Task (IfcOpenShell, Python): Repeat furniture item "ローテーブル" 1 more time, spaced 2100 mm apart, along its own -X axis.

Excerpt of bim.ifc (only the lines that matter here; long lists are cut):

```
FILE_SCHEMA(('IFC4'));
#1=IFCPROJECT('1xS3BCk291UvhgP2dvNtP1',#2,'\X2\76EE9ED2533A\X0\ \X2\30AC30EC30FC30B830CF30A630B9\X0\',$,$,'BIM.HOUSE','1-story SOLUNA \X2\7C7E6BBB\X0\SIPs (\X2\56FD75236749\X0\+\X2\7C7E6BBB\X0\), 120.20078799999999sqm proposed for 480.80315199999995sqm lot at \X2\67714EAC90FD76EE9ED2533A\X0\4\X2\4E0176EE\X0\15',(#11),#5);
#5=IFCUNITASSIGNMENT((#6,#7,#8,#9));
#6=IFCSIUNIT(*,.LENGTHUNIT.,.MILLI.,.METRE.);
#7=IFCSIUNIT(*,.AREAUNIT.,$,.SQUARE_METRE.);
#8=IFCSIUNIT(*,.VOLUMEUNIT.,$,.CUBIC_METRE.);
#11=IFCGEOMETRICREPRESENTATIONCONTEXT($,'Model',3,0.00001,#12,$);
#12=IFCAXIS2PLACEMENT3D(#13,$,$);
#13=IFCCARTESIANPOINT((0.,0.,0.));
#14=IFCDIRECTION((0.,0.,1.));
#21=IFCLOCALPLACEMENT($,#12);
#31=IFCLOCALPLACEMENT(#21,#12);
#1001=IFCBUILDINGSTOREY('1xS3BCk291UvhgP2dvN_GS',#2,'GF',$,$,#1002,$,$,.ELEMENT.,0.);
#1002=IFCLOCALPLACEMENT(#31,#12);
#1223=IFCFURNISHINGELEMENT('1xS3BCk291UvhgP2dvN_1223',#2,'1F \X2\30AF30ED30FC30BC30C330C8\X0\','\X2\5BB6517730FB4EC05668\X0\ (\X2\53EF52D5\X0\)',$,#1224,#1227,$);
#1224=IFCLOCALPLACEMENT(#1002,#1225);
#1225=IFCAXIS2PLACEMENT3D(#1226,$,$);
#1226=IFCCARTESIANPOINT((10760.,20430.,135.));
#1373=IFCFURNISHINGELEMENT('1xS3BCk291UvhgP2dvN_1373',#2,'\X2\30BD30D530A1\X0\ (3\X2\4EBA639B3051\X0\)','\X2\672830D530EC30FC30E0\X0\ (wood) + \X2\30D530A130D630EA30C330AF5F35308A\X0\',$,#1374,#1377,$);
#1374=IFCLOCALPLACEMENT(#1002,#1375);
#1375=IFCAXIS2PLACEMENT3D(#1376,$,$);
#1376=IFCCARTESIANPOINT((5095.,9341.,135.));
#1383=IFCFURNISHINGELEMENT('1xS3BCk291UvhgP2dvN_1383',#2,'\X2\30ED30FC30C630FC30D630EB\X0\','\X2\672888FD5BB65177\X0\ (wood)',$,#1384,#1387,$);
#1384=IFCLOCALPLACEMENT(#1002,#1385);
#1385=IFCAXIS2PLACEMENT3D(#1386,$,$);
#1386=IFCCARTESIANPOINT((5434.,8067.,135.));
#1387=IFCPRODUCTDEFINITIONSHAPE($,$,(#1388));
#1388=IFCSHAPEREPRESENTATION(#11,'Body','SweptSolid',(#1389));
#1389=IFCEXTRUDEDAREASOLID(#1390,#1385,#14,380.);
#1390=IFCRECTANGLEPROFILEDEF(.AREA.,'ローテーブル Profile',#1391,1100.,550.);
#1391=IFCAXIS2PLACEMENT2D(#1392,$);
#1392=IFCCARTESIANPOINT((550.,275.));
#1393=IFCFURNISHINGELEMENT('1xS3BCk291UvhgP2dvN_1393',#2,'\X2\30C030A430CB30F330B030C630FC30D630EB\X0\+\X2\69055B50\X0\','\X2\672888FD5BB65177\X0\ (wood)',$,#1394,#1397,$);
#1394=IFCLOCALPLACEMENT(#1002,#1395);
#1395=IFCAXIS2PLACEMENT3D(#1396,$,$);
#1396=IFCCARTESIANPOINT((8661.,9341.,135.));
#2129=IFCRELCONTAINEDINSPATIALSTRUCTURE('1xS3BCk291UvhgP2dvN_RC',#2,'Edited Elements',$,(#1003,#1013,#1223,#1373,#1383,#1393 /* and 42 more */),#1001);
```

```python
import ifcopenshell
import ifcopenshell.api.geometry
import ifcopenshell.api.root
import ifcopenshell.util.element
import ifcopenshell.util.placement
import ifcopenshell.util.unit

model = ifcopenshell.open("bim.ifc")
unit_scale = ifcopenshell.util.unit.calculate_unit_scale(model)


def reuse_history(source, copy):
    """copy_class also copies each property set's owner history, people and application; keep the originals."""
    for rel in copy.IsDefinedBy:
        if rel.is_a("IfcRelDefinesByProperties") and (history := rel.RelatingPropertyDefinition.OwnerHistory):
            rel.RelatingPropertyDefinition.OwnerHistory = source.OwnerHistory
            ifcopenshell.util.element.remove_deep2(model, history)


source = model.by_guid("1xS3BCk291UvhgP2dvN_1383")
base = ifcopenshell.util.placement.get_local_placement(source.ObjectPlacement)
step = -base[:3, 0] * 2.1 / unit_scale

for i in range(1, 2):
    copy = ifcopenshell.api.root.copy_class(model, product=source)
    copy.Representation = ifcopenshell.util.element.copy_deep(
        model, source.Representation, exclude=["IfcGeometricRepresentationContext", "IfcRepresentationMap"]
    )
    reuse_history(source, copy)
    matrix = base.copy()
    matrix[:3, 3] += i * step
    print("added at", matrix[:3, 3].round(3) + 0.0)
    ifcopenshell.api.geometry.edit_object_placement(model, product=copy, matrix=matrix, is_si=False)

model.write("bim_rev.ifc")
```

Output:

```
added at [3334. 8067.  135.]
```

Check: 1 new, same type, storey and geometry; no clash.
